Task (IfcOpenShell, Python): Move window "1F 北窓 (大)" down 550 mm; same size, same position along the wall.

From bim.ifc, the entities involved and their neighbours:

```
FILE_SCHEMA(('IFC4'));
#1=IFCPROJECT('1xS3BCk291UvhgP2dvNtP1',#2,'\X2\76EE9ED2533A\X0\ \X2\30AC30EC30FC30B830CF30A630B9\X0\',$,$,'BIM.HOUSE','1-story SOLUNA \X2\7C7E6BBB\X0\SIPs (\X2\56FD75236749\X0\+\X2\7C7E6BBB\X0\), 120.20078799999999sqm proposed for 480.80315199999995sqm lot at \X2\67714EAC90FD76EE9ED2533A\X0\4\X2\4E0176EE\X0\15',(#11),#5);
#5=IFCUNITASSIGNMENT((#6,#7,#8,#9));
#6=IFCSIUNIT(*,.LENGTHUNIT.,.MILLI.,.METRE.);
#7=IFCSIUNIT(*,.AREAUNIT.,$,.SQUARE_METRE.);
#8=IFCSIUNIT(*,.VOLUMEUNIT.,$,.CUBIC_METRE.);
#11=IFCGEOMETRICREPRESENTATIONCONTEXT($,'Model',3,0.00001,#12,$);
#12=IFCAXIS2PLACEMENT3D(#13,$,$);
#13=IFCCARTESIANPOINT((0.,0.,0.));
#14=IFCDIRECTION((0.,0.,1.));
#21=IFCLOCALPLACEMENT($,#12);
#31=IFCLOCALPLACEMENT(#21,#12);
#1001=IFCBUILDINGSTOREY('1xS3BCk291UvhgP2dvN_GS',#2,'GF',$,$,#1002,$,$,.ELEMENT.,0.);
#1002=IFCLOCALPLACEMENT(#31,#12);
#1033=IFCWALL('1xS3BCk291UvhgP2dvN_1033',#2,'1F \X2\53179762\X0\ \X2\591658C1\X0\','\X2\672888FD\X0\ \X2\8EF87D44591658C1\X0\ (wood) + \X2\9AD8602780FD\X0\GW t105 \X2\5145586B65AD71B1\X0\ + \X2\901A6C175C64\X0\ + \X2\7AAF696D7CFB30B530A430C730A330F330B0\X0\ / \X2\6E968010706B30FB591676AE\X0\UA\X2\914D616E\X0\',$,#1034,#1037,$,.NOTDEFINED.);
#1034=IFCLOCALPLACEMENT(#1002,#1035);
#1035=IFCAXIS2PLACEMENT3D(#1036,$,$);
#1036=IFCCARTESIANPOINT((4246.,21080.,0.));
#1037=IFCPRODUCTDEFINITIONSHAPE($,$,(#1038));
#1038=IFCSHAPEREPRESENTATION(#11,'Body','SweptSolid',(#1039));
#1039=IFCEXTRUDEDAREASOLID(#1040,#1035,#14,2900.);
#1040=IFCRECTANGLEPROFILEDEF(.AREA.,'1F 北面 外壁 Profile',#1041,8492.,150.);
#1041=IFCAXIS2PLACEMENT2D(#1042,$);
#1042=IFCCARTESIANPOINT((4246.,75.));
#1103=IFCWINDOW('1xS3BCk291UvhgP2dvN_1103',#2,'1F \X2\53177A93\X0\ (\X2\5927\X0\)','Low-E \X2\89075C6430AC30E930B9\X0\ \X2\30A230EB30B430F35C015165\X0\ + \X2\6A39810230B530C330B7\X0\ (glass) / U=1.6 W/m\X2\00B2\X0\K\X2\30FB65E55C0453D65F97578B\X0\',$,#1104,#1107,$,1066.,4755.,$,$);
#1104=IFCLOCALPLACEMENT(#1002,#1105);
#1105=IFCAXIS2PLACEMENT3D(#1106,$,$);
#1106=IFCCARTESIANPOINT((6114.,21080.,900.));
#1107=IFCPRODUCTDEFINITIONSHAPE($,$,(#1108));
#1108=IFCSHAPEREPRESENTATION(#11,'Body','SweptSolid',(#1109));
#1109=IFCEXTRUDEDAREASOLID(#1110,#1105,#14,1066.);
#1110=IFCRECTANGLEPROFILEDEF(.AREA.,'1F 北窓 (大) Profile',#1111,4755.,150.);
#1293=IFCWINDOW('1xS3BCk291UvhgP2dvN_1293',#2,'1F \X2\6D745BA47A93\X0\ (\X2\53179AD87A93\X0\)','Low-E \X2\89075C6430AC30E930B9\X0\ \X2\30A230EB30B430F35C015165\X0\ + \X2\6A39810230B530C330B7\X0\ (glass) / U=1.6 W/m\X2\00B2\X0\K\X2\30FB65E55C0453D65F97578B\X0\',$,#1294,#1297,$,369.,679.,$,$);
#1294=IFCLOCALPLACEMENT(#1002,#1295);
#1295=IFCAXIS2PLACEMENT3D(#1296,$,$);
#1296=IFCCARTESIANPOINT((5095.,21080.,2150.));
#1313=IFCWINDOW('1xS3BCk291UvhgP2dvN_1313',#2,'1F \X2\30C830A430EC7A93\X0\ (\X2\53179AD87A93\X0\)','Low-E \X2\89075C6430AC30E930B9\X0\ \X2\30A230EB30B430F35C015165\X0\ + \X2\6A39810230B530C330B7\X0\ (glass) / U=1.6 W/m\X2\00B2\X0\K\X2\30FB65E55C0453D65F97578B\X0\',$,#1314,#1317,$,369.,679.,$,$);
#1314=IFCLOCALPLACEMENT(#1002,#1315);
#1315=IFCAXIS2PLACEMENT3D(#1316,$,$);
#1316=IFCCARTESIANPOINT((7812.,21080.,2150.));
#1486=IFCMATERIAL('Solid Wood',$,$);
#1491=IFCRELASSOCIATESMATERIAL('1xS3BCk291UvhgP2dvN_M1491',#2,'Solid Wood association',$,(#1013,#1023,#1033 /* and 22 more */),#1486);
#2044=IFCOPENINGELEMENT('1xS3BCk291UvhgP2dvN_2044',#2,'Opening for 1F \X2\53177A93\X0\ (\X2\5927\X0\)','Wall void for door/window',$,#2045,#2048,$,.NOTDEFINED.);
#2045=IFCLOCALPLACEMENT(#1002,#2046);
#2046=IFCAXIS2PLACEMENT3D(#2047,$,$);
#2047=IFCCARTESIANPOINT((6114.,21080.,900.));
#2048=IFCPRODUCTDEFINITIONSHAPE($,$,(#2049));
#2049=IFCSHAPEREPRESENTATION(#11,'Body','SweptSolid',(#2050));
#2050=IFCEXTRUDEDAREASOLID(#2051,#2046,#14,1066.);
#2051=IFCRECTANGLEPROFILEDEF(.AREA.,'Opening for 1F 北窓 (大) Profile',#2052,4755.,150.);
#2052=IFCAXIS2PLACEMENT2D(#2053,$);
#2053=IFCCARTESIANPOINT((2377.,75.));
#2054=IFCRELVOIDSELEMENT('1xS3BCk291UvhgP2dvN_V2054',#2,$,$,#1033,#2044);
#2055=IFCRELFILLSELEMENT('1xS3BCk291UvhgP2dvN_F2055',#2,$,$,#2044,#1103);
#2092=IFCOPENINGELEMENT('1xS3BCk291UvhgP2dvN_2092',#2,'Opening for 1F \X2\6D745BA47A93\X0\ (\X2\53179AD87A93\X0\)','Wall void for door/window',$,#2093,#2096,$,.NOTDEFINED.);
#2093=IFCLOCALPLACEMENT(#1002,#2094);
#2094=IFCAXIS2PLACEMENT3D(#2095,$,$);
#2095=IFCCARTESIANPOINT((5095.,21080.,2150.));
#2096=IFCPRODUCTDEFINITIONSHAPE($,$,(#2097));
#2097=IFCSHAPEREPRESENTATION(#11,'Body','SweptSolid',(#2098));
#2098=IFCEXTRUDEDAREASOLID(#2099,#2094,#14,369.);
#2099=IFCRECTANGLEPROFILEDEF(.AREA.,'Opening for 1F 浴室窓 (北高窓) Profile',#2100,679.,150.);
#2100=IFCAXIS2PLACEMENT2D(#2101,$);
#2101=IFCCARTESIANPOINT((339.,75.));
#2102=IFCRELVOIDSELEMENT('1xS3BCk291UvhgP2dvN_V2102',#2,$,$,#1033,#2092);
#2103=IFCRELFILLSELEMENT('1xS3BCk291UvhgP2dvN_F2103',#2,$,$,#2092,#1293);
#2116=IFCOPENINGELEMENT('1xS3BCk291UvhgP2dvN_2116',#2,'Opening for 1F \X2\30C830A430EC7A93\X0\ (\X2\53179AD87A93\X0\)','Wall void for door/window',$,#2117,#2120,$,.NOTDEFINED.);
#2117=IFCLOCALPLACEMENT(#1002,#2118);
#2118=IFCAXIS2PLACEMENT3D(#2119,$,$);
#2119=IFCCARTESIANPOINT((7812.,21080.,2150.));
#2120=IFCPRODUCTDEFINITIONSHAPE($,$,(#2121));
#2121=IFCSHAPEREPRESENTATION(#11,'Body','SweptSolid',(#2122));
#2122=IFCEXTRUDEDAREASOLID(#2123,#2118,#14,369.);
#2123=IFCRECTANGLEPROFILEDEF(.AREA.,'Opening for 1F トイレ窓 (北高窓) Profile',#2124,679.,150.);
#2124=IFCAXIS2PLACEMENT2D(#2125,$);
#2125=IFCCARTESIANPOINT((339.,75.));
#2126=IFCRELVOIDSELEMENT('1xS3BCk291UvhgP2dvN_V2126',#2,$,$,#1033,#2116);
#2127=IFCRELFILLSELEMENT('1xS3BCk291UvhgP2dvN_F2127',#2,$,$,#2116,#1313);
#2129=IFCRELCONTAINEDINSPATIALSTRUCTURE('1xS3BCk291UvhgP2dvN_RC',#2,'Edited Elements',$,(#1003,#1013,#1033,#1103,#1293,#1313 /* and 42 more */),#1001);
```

```python
import numpy as np
import ifcopenshell
import ifcopenshell.api.geometry
import ifcopenshell.util.placement
import ifcopenshell.util.unit

model = ifcopenshell.open("bim.ifc")
unit_scale = ifcopenshell.util.unit.calculate_unit_scale(model)

window = model.by_id(1103)
opening = window.FillsVoids[0].RelatingOpeningElement
dz = -550.0

shift = np.array([0.0, 0.0, dz])
# The window is not placed relative to its opening, so move both.
for product in (opening, window):
    matrix = ifcopenshell.util.placement.get_local_placement(product.ObjectPlacement)
    matrix[:3, 3] += shift
    ifcopenshell.api.geometry.edit_object_placement(model, product=product, matrix=matrix, is_si=False)

print(f"moved by {dz * unit_scale:+.3f} m")

model.write("bim_rev.ifc")
```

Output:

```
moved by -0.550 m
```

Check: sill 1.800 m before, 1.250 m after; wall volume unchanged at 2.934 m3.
